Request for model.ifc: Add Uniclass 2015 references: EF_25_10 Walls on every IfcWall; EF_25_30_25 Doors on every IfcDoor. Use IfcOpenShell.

First a look at what the model holds.

```python
import ifcopenshell

model = ifcopenshell.open("model.ifc")
print(model.schema)
print("classifications:", [c.Name for c in model.by_type("IfcClassification")])
for ifc_class in ("IfcDoor", "IfcRoof", "IfcStair", "IfcWall", "IfcWindow"):
    print(ifc_class, len(model.by_type(ifc_class)))
```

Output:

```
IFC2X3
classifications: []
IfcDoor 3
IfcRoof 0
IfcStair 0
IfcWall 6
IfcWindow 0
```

```python
import ifcopenshell
import ifcopenshell.api.classification

model = ifcopenshell.open("model.ifc")

# IFC2X3 requires Source and Edition and has no link from the project to the system.
system = model.create_entity("IfcClassification", Source="NBS", Edition="2015", Name="Uniclass 2015")

codes = {
    "IfcWall": ("EF_25_10", "Walls"),
    "IfcDoor": ("EF_25_30_25", "Doors"),
}
for ifc_class, (code, name) in codes.items():
    products = model.by_type(ifc_class)
    ifcopenshell.api.classification.add_reference(
        model, products=products, classification=system, identification=code, name=name
    )
    print(code, len(products))

model.write("model_updated.ifc")
```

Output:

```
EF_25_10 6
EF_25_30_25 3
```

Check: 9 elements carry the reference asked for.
